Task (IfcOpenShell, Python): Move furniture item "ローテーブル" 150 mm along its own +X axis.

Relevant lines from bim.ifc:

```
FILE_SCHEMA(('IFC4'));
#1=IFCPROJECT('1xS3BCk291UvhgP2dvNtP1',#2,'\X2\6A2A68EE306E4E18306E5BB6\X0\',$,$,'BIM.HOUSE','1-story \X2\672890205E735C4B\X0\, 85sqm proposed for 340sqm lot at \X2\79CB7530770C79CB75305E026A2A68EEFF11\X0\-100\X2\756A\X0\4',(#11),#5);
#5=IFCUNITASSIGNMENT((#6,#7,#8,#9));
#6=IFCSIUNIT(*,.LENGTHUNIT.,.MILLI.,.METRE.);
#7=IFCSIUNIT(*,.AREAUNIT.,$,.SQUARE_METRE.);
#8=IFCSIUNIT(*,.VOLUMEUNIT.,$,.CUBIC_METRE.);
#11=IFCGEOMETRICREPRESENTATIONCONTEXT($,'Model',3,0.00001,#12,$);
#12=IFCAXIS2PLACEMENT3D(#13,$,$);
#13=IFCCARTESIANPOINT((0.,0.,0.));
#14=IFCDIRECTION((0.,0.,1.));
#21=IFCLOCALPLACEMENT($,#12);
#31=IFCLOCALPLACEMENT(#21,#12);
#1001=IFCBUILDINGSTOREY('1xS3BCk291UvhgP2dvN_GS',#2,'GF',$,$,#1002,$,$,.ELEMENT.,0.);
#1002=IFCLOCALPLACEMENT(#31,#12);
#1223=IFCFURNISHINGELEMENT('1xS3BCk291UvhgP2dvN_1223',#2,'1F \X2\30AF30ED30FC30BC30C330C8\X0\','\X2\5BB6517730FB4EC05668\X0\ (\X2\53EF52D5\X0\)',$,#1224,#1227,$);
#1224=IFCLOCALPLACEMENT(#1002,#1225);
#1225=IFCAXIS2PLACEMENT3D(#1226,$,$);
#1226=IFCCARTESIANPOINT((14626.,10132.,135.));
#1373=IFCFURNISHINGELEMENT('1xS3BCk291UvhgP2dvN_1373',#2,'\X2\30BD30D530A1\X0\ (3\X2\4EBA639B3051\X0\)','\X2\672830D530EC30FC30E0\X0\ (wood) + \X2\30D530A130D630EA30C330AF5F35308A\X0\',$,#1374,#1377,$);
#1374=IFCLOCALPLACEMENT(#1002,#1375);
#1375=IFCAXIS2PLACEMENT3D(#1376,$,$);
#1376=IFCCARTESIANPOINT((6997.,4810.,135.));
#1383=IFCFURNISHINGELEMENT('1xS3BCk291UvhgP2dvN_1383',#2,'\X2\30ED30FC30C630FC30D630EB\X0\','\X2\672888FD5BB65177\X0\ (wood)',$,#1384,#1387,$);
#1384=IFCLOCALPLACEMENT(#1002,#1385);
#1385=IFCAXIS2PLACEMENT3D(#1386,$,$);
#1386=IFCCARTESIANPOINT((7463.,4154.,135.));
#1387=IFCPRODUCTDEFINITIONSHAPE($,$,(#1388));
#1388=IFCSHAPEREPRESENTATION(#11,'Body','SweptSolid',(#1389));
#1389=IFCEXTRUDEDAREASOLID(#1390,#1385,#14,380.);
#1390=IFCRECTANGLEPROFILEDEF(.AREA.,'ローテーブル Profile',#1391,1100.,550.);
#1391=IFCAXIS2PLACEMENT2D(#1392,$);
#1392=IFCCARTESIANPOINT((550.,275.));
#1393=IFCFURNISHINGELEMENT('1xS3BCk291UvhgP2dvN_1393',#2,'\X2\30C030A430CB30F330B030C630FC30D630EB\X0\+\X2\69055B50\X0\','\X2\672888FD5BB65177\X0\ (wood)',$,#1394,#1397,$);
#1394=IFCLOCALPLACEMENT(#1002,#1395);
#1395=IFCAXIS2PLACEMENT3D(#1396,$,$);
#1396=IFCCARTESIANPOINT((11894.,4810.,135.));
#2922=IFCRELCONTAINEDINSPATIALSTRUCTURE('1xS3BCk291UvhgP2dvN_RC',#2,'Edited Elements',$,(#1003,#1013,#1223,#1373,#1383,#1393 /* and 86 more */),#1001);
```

```python
import ifcopenshell
import ifcopenshell.api.geometry
import ifcopenshell.util.placement

model = ifcopenshell.open("bim.ifc")

item = model.by_guid("1xS3BCk291UvhgP2dvN_1383")
matrix = ifcopenshell.util.placement.get_local_placement(item.ObjectPlacement)
matrix[:3, 3] += matrix[:3, 0] * 150.0
ifcopenshell.api.geometry.edit_object_placement(model, product=item, matrix=matrix, is_si=False)

print(ifcopenshell.util.placement.get_local_placement(item.ObjectPlacement).round(3) + 0.0)

model.write("bim_updated.ifc")
```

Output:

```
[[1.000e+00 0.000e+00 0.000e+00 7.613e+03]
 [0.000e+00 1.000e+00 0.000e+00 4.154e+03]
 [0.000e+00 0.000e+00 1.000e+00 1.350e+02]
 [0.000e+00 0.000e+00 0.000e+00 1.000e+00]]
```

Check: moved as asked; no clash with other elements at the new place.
